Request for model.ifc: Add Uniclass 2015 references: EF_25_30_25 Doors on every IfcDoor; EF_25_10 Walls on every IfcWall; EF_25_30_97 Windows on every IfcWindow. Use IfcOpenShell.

First a look at what the model holds.

```python
import ifcopenshell

model = ifcopenshell.open("model.ifc")
print(model.schema)
print("classifications:", [c.Name for c in model.by_type("IfcClassification")])
for ifc_class in ("IfcDoor", "IfcRoof", "IfcStair", "IfcWall", "IfcWindow"):
    print(ifc_class, len(model.by_type(ifc_class)))
```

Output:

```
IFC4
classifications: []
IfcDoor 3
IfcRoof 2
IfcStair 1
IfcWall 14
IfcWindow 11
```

```python
import ifcopenshell
import ifcopenshell.api.classification

model = ifcopenshell.open("model.ifc")

system = ifcopenshell.api.classification.add_classification(model, classification="Uniclass 2015")

codes = {
    "IfcDoor": ("EF_25_30_25", "Doors"),
    "IfcWall": ("EF_25_10", "Walls"),
    "IfcWindow": ("EF_25_30_97", "Windows"),
}
for ifc_class, (code, name) in codes.items():
    products = model.by_type(ifc_class)
    ifcopenshell.api.classification.add_reference(
        model, products=products, classification=system, identification=code, name=name
    )
    print(code, len(products))

model.write("model_updated.ifc")
```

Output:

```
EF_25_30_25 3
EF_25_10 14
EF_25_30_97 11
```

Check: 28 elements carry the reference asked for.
